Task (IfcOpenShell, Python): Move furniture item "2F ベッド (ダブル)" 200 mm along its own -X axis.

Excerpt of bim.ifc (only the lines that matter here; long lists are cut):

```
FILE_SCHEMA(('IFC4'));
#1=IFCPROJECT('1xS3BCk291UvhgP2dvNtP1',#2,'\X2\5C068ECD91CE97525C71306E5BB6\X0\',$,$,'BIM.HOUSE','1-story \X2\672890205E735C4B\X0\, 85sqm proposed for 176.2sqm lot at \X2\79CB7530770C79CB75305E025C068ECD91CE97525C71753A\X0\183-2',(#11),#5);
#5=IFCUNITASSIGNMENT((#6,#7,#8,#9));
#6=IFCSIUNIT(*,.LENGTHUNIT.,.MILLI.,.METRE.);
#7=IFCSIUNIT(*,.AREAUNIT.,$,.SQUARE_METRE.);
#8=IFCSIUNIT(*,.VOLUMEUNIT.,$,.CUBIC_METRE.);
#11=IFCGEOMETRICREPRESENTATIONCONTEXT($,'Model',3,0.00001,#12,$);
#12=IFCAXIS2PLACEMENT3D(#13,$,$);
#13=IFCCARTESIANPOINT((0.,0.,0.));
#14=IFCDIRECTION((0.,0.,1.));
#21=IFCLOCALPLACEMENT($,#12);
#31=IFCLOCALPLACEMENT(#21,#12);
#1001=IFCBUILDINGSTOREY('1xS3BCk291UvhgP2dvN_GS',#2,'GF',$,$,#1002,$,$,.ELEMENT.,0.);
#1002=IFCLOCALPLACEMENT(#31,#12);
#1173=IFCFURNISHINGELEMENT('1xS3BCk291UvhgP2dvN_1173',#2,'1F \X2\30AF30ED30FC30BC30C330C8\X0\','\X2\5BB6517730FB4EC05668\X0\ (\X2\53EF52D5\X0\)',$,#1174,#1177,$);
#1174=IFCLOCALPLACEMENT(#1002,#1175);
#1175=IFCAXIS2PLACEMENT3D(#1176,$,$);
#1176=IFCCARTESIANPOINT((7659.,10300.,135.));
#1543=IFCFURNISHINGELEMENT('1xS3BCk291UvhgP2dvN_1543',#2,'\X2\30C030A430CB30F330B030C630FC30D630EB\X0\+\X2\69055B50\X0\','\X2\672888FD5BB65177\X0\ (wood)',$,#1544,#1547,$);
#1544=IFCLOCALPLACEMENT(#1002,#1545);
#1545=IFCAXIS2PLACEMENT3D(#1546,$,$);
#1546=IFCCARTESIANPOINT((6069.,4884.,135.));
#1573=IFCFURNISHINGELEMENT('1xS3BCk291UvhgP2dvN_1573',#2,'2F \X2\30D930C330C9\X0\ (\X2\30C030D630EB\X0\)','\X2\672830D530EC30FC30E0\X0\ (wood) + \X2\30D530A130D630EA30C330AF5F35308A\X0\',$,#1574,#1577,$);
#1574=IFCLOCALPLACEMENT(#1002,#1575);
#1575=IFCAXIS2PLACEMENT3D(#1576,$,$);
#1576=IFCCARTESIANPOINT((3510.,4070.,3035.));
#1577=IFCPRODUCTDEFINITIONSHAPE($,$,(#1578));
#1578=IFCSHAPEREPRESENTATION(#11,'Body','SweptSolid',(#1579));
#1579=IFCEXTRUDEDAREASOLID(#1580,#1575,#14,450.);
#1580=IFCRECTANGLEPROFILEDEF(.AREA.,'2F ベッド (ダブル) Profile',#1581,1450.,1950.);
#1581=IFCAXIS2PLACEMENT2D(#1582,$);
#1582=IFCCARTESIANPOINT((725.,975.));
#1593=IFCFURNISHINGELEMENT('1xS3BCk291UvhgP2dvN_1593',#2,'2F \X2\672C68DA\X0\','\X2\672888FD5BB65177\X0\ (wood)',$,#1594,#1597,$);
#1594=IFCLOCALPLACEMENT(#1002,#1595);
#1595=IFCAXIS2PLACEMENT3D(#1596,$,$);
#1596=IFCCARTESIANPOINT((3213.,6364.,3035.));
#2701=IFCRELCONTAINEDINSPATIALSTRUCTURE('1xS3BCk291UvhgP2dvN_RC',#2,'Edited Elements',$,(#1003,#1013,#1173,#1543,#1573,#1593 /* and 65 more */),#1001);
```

```python
import ifcopenshell
import ifcopenshell.api.geometry
import ifcopenshell.util.placement

model = ifcopenshell.open("bim.ifc")

item = model.by_guid("1xS3BCk291UvhgP2dvN_1573")
matrix = ifcopenshell.util.placement.get_local_placement(item.ObjectPlacement)
matrix[:3, 3] -= matrix[:3, 0] * 200.0
ifcopenshell.api.geometry.edit_object_placement(model, product=item, matrix=matrix, is_si=False)

print(ifcopenshell.util.placement.get_local_placement(item.ObjectPlacement).round(3) + 0.0)

model.write("bim_updated.ifc")
```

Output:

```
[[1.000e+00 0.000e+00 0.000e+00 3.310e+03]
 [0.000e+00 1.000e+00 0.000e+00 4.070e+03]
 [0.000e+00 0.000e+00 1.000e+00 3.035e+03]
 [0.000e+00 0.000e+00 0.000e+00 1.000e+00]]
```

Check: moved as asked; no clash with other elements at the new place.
